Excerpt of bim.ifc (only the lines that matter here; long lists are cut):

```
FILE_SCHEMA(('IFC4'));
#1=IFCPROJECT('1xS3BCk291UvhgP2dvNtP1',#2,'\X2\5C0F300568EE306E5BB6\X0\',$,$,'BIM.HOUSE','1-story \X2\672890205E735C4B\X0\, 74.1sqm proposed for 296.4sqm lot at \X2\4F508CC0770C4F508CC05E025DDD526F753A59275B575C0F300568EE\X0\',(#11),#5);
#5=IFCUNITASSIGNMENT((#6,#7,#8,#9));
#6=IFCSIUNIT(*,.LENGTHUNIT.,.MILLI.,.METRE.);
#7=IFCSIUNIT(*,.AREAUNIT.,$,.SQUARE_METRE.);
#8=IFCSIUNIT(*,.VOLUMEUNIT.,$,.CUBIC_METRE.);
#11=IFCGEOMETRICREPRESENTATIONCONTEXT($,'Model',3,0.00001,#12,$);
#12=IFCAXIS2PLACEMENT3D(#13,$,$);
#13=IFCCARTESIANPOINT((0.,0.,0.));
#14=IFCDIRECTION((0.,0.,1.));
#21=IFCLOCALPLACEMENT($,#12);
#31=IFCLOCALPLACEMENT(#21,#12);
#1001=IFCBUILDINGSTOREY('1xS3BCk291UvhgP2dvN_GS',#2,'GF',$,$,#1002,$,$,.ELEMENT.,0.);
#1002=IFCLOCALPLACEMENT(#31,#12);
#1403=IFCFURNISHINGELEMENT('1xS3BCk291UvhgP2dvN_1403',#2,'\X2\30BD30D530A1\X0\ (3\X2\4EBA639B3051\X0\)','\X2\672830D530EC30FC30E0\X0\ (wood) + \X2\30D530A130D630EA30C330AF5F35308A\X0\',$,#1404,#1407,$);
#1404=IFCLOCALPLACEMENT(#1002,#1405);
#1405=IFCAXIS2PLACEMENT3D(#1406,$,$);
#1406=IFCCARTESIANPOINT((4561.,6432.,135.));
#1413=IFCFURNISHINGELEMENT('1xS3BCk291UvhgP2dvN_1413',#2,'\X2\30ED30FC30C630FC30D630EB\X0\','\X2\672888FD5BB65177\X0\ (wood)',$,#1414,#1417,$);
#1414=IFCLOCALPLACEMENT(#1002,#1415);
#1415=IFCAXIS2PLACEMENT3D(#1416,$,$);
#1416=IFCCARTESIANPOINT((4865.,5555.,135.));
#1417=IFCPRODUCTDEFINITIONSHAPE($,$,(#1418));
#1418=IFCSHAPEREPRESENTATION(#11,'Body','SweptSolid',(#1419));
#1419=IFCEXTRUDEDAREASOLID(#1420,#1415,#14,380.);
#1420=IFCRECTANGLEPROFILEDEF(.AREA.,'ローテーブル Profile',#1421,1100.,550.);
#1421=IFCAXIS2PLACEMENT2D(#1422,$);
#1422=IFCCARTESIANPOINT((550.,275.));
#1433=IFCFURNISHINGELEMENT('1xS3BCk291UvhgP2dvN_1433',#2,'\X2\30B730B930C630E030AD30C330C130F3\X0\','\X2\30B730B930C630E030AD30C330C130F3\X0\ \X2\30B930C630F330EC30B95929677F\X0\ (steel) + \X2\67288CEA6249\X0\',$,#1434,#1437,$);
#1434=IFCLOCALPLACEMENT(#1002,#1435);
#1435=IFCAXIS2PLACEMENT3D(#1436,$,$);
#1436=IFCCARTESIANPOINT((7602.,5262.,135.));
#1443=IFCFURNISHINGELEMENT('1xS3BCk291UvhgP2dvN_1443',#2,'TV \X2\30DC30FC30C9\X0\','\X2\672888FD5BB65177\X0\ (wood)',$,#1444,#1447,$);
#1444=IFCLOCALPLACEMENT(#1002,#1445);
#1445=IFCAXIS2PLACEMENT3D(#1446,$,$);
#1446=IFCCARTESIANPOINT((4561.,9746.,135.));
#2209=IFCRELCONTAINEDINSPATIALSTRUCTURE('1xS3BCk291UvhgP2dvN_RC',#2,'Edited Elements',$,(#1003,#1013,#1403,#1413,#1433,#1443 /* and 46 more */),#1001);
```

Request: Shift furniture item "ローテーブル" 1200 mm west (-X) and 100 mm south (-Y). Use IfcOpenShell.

```python
import ifcopenshell
import ifcopenshell.api.geometry
import ifcopenshell.util.placement
import ifcopenshell.util.unit

model = ifcopenshell.open("bim.ifc")
unit_scale = ifcopenshell.util.unit.calculate_unit_scale(model)

item = model.by_guid("1xS3BCk291UvhgP2dvN_1413")
matrix = ifcopenshell.util.placement.get_local_placement(item.ObjectPlacement)
matrix[0, 3] -= 1.2 / unit_scale
matrix[1, 3] -= 0.1 / unit_scale
ifcopenshell.api.geometry.edit_object_placement(model, product=item, matrix=matrix, is_si=False)

print(ifcopenshell.util.placement.get_local_placement(item.ObjectPlacement).round(3) + 0.0)

model.write("bim_edited.ifc")
```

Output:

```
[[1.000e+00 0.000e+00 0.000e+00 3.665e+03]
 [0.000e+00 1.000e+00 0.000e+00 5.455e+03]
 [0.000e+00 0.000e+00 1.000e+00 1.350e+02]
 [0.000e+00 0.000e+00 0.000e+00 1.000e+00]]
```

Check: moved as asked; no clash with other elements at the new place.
